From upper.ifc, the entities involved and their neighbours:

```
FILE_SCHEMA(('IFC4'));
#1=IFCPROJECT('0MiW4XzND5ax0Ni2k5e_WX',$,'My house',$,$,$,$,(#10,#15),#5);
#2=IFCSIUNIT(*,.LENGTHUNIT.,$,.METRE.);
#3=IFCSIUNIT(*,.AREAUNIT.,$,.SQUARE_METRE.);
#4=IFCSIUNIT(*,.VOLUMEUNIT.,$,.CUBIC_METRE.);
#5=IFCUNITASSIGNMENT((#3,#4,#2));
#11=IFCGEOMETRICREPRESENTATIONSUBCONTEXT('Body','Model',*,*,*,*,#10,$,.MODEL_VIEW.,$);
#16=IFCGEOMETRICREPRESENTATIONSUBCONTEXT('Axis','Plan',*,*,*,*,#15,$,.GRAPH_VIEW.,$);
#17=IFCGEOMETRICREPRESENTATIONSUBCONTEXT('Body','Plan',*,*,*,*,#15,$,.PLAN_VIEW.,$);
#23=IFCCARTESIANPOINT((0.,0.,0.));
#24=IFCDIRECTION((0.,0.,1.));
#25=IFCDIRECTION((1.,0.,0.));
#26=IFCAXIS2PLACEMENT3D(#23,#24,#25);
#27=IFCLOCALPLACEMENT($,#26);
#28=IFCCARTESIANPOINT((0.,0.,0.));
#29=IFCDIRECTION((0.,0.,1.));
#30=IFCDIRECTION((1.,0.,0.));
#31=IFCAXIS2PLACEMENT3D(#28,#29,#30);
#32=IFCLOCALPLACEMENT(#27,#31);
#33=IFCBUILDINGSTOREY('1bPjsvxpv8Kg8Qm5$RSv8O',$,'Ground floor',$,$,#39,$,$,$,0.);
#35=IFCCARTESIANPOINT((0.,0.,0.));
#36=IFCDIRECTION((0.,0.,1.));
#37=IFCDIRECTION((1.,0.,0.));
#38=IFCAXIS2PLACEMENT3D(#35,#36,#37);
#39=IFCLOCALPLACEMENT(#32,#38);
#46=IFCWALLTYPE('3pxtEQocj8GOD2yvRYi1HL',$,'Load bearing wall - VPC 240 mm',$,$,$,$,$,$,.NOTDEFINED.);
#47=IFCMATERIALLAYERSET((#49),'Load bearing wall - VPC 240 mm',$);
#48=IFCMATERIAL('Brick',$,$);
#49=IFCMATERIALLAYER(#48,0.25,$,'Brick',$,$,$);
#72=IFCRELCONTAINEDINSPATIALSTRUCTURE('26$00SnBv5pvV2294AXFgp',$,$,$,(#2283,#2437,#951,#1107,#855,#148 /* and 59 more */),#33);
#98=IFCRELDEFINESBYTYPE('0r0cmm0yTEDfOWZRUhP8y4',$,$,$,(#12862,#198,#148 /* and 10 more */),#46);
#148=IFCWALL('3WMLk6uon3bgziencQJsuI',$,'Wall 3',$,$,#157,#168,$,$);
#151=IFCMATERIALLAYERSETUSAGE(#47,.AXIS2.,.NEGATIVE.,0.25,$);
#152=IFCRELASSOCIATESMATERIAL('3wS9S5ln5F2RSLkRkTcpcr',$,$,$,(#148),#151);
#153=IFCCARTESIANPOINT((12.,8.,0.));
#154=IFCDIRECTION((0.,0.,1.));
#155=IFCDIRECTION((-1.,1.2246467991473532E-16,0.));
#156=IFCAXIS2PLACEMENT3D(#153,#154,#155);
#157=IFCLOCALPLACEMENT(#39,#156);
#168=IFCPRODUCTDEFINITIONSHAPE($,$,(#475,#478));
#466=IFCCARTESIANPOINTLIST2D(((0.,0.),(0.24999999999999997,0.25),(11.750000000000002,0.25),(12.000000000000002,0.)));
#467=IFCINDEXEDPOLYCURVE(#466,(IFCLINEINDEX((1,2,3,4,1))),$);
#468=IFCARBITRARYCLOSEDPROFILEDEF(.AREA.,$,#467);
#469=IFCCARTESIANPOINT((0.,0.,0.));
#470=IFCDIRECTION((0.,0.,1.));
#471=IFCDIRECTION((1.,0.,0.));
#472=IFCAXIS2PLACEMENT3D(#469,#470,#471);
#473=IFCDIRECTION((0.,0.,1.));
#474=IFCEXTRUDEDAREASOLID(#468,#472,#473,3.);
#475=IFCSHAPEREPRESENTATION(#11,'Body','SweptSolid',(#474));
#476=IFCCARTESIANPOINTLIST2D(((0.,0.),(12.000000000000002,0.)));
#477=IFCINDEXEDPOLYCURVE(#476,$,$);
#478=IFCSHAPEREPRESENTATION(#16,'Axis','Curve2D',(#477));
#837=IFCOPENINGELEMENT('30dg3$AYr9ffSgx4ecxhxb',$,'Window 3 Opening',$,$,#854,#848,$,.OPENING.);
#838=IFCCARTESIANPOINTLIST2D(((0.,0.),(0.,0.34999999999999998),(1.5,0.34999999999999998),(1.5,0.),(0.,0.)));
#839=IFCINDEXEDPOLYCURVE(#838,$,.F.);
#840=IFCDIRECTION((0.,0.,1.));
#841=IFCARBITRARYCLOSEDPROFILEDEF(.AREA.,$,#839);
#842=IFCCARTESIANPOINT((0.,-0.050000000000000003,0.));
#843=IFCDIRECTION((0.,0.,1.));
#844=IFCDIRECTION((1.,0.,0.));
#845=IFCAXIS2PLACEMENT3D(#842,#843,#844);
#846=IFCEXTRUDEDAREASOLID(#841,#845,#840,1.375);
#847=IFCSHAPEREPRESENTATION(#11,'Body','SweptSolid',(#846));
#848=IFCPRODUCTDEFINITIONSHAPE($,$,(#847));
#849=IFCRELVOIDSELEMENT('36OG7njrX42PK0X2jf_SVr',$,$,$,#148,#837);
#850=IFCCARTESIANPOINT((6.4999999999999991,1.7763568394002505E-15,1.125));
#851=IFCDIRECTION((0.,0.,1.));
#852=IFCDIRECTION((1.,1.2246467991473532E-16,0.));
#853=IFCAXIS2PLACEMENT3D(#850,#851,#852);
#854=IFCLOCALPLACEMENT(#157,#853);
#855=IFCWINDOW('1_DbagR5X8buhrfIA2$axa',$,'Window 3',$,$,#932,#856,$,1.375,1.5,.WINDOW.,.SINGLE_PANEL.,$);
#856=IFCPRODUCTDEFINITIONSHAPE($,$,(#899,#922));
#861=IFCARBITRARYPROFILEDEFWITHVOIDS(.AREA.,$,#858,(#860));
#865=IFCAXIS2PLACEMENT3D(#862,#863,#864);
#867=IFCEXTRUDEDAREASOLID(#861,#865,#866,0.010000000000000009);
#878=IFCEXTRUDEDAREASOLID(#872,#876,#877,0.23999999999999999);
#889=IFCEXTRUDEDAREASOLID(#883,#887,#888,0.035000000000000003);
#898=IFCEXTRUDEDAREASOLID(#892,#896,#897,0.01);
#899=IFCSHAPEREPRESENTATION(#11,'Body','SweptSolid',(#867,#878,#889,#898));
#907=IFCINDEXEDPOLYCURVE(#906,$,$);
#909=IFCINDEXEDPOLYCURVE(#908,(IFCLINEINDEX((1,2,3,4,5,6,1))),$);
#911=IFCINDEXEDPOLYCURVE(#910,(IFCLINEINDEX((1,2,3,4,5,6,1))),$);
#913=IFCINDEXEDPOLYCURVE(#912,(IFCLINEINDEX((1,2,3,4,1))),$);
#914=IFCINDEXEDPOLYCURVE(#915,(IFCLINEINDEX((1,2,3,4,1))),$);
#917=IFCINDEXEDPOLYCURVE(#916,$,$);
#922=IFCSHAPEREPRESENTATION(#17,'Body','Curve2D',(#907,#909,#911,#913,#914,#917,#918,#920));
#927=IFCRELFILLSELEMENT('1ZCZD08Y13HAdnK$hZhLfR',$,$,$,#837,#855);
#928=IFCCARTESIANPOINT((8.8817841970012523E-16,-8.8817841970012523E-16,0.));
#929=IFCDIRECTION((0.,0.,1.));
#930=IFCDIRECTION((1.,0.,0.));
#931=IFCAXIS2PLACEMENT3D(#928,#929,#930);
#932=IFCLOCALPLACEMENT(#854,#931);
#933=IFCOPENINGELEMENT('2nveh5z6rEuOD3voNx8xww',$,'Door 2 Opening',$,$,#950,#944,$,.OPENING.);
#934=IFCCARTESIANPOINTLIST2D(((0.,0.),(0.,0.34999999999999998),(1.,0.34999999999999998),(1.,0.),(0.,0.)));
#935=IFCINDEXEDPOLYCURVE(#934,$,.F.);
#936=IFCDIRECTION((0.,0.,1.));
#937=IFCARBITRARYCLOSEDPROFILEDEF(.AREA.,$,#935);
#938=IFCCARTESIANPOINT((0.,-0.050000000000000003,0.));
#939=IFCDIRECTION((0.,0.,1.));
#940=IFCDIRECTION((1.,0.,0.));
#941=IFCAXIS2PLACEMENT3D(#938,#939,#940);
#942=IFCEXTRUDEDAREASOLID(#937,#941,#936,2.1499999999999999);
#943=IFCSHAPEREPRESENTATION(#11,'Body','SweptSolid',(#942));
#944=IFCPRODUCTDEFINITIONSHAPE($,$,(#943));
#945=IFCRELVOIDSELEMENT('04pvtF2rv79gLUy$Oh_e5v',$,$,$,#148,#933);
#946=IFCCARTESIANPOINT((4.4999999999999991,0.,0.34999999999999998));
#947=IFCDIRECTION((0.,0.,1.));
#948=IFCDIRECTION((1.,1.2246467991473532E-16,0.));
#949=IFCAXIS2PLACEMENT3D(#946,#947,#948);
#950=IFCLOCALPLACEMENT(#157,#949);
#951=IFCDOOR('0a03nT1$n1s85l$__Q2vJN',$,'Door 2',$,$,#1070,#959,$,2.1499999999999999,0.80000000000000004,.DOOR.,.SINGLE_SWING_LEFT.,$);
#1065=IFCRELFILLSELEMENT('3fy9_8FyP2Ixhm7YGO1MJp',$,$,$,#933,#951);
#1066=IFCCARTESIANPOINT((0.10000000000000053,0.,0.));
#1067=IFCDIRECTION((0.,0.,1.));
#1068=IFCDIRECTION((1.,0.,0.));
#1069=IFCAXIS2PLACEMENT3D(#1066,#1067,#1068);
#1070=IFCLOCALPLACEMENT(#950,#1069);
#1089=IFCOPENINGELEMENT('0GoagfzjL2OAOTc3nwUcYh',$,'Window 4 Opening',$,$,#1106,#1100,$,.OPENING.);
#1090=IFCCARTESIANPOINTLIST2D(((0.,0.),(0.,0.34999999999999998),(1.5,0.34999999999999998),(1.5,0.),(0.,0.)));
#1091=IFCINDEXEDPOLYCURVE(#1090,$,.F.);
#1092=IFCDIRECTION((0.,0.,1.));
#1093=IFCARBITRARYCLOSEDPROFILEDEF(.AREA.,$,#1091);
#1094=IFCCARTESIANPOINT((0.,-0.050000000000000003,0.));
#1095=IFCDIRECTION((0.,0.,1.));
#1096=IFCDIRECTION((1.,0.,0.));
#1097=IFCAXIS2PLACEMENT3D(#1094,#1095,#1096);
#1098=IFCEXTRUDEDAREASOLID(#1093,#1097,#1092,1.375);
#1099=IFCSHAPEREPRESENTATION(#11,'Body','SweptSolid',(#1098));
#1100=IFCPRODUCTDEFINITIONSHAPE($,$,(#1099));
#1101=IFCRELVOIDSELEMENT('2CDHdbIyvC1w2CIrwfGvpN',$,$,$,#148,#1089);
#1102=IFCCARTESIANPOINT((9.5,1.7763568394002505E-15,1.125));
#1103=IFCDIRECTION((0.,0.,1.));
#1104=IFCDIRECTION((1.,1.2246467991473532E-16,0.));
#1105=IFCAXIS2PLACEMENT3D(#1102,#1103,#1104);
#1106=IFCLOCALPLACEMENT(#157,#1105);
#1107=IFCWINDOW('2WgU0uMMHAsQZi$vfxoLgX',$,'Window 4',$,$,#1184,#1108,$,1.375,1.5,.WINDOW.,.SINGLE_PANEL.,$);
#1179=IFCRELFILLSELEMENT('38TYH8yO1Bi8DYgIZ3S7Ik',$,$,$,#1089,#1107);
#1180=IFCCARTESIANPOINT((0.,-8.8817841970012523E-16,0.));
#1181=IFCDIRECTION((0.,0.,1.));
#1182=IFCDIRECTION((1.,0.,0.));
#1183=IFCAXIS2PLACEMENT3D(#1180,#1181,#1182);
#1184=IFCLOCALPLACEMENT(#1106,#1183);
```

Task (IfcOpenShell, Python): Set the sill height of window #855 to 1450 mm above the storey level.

```python
import numpy as np
import ifcopenshell
import ifcopenshell.api.geometry
import ifcopenshell.geom
import ifcopenshell.util.element
import ifcopenshell.util.placement
import ifcopenshell.util.shape
import ifcopenshell.util.unit

model = ifcopenshell.open("upper.ifc")
unit_scale = ifcopenshell.util.unit.calculate_unit_scale(model)

window = model.by_id(855)
opening = window.FillsVoids[0].RelatingOpeningElement
storey = ifcopenshell.util.element.get_container(window, ifc_class="IfcBuildingStorey")
level = ifcopenshell.util.placement.get_local_placement(storey.ObjectPlacement)[2, 3]

# The opening's origin need not be at the sill, so measure its lowest point.
shape = ifcopenshell.geom.create_shape(ifcopenshell.geom.settings(), opening)
bottom = ifcopenshell.util.shape.get_shape_bottom_elevation(shape, shape.geometry) / unit_scale
dz = level + 1.45 / unit_scale - bottom

shift = np.array([0.0, 0.0, dz])
# The window is placed relative to its opening, so it follows when the opening moves.
matrix = ifcopenshell.util.placement.get_local_placement(opening.ObjectPlacement)
matrix[:3, 3] += shift
ifcopenshell.api.geometry.edit_object_placement(
    model, product=opening, matrix=matrix, is_si=False, should_transform_children=True
)

print(f"moved by {dz * unit_scale:+.3f} m")

model.write("upper_rev.ifc")
```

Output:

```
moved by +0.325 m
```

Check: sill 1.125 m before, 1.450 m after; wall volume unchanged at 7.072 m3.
